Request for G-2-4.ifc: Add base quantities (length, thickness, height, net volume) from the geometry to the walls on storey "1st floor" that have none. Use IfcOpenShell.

First a look at what the model holds.

```python
import ifcopenshell
import ifcopenshell.util.element
import ifcopenshell.util.unit

model = ifcopenshell.open("G-2-4.ifc")
print(model.schema)
for unit_type in ("LENGTHUNIT", "AREAUNIT", "VOLUMEUNIT"):
    print(unit_type, ifcopenshell.util.unit.calculate_unit_scale(model, unit_type))
storey = next(s for s in model.by_type("IfcBuildingStorey") if s.Name == "1st floor")
walls = [e for e in ifcopenshell.util.element.get_decomposition(storey) if e.is_a("IfcWall")]
for e in sorted(walls, key=lambda e: e.id()):
    print(e.id(), e.is_a(), e.Name, list(ifcopenshell.util.element.get_psets(e, qtos_only=True)), sep=" | ")
```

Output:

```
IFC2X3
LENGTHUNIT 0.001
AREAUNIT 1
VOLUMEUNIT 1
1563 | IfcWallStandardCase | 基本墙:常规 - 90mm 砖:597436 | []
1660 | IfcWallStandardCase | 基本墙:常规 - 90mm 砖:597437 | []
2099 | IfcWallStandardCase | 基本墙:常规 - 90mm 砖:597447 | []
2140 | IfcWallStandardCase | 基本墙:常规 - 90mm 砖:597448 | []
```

```python
import ifcopenshell
import ifcopenshell.api.pset
import ifcopenshell.geom
import ifcopenshell.util.element
import ifcopenshell.util.shape
import ifcopenshell.util.unit

model = ifcopenshell.open("G-2-4.ifc")
unit_scale = ifcopenshell.util.unit.calculate_unit_scale(model)
volume_scale = ifcopenshell.util.unit.calculate_unit_scale(model, "VOLUMEUNIT")
settings = ifcopenshell.geom.settings()

storey = next(s for s in model.by_type("IfcBuildingStorey") if s.Name == "1st floor")
walls = [e for e in ifcopenshell.util.element.get_decomposition(storey) if e.is_a("IfcWall")]

for e in sorted(walls, key=lambda e: e.id()):
    if ifcopenshell.util.element.get_psets(e, qtos_only=True, should_inherit=False):
        continue
    # Geometry comes back in metres, in the element's own axes.
    shape = ifcopenshell.geom.create_shape(settings, e)
    values = {
        "Length": ifcopenshell.util.shape.get_x(shape.geometry) / unit_scale,
        "Width": ifcopenshell.util.shape.get_y(shape.geometry) / unit_scale,
        "Height": ifcopenshell.util.shape.get_z(shape.geometry) / unit_scale,
        "NetVolume": ifcopenshell.util.shape.get_volume(shape.geometry) / volume_scale,
    }
    qto = ifcopenshell.api.pset.add_qto(model, product=e, name="BaseQuantities")
    ifcopenshell.api.pset.edit_qto(model, qto=qto, properties=values)
    print(e.id(), {k: round(v, 3) for k, v in values.items()})

model.write("G-2-4-out.ifc")
```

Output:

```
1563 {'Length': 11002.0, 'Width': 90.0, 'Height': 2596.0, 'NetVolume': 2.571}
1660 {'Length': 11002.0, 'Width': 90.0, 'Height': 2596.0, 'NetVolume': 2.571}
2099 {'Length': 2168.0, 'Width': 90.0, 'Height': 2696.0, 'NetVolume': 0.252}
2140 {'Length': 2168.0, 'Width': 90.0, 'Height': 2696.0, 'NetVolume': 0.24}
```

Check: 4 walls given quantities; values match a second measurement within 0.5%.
